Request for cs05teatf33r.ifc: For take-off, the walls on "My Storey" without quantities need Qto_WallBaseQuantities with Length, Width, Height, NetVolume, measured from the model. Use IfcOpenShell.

First a look at what the model holds.

```python
import ifcopenshell
import ifcopenshell.util.element
import ifcopenshell.util.unit

model = ifcopenshell.open("cs05teatf33r.ifc")
print(model.schema)
for unit_type in ("LENGTHUNIT", "AREAUNIT", "VOLUMEUNIT"):
    print(unit_type, ifcopenshell.util.unit.calculate_unit_scale(model, unit_type))
storey = next(s for s in model.by_type("IfcBuildingStorey") if s.Name == "My Storey")
walls = [e for e in ifcopenshell.util.element.get_decomposition(storey) if e.is_a("IfcWall")]
for e in sorted(walls, key=lambda e: e.id()):
    print(e.id(), e.is_a(), e.Name, list(ifcopenshell.util.element.get_psets(e, qtos_only=True)), sep=" | ")
```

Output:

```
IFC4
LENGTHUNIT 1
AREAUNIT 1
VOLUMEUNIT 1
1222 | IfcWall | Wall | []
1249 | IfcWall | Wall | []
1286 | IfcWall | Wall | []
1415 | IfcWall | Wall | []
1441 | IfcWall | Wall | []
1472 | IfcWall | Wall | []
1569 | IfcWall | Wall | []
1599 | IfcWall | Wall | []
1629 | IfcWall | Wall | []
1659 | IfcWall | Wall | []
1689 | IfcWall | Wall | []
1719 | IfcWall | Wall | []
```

```python
import ifcopenshell
import ifcopenshell.api.pset
import ifcopenshell.geom
import ifcopenshell.util.element
import ifcopenshell.util.shape
import ifcopenshell.util.unit

model = ifcopenshell.open("cs05teatf33r.ifc")
unit_scale = ifcopenshell.util.unit.calculate_unit_scale(model)
volume_scale = ifcopenshell.util.unit.calculate_unit_scale(model, "VOLUMEUNIT")
settings = ifcopenshell.geom.settings()

storey = next(s for s in model.by_type("IfcBuildingStorey") if s.Name == "My Storey")
walls = [e for e in ifcopenshell.util.element.get_decomposition(storey) if e.is_a("IfcWall")]

for e in sorted(walls, key=lambda e: e.id()):
    if ifcopenshell.util.element.get_psets(e, qtos_only=True, should_inherit=False):
        continue
    # Geometry comes back in metres, in the element's own axes.
    shape = ifcopenshell.geom.create_shape(settings, e)
    values = {
        "Length": ifcopenshell.util.shape.get_x(shape.geometry) / unit_scale,
        "Width": ifcopenshell.util.shape.get_y(shape.geometry) / unit_scale,
        "Height": ifcopenshell.util.shape.get_z(shape.geometry) / unit_scale,
        "NetVolume": ifcopenshell.util.shape.get_volume(shape.geometry) / volume_scale,
    }
    qto = ifcopenshell.api.pset.add_qto(model, product=e, name="Qto_WallBaseQuantities")
    ifcopenshell.api.pset.edit_qto(model, qto=qto, properties=values)
    print(e.id(), {k: round(v, 3) for k, v in values.items()})

model.write("cs05teatf33r-out.ifc")
```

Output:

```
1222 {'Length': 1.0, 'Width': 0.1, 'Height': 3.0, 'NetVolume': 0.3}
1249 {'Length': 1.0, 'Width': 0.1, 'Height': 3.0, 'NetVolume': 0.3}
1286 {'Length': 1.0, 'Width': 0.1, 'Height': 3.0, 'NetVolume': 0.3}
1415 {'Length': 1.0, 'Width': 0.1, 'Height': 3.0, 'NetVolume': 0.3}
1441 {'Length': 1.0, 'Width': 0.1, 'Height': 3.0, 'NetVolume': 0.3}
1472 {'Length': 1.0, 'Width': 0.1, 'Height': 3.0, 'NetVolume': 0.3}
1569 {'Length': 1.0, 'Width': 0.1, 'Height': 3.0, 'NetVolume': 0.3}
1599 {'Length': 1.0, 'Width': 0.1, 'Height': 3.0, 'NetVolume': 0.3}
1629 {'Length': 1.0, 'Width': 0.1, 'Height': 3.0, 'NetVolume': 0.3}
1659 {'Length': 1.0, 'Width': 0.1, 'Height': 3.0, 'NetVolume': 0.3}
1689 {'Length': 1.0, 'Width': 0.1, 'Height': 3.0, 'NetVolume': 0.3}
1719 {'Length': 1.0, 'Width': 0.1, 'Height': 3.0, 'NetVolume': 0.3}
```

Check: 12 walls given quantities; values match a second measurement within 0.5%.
